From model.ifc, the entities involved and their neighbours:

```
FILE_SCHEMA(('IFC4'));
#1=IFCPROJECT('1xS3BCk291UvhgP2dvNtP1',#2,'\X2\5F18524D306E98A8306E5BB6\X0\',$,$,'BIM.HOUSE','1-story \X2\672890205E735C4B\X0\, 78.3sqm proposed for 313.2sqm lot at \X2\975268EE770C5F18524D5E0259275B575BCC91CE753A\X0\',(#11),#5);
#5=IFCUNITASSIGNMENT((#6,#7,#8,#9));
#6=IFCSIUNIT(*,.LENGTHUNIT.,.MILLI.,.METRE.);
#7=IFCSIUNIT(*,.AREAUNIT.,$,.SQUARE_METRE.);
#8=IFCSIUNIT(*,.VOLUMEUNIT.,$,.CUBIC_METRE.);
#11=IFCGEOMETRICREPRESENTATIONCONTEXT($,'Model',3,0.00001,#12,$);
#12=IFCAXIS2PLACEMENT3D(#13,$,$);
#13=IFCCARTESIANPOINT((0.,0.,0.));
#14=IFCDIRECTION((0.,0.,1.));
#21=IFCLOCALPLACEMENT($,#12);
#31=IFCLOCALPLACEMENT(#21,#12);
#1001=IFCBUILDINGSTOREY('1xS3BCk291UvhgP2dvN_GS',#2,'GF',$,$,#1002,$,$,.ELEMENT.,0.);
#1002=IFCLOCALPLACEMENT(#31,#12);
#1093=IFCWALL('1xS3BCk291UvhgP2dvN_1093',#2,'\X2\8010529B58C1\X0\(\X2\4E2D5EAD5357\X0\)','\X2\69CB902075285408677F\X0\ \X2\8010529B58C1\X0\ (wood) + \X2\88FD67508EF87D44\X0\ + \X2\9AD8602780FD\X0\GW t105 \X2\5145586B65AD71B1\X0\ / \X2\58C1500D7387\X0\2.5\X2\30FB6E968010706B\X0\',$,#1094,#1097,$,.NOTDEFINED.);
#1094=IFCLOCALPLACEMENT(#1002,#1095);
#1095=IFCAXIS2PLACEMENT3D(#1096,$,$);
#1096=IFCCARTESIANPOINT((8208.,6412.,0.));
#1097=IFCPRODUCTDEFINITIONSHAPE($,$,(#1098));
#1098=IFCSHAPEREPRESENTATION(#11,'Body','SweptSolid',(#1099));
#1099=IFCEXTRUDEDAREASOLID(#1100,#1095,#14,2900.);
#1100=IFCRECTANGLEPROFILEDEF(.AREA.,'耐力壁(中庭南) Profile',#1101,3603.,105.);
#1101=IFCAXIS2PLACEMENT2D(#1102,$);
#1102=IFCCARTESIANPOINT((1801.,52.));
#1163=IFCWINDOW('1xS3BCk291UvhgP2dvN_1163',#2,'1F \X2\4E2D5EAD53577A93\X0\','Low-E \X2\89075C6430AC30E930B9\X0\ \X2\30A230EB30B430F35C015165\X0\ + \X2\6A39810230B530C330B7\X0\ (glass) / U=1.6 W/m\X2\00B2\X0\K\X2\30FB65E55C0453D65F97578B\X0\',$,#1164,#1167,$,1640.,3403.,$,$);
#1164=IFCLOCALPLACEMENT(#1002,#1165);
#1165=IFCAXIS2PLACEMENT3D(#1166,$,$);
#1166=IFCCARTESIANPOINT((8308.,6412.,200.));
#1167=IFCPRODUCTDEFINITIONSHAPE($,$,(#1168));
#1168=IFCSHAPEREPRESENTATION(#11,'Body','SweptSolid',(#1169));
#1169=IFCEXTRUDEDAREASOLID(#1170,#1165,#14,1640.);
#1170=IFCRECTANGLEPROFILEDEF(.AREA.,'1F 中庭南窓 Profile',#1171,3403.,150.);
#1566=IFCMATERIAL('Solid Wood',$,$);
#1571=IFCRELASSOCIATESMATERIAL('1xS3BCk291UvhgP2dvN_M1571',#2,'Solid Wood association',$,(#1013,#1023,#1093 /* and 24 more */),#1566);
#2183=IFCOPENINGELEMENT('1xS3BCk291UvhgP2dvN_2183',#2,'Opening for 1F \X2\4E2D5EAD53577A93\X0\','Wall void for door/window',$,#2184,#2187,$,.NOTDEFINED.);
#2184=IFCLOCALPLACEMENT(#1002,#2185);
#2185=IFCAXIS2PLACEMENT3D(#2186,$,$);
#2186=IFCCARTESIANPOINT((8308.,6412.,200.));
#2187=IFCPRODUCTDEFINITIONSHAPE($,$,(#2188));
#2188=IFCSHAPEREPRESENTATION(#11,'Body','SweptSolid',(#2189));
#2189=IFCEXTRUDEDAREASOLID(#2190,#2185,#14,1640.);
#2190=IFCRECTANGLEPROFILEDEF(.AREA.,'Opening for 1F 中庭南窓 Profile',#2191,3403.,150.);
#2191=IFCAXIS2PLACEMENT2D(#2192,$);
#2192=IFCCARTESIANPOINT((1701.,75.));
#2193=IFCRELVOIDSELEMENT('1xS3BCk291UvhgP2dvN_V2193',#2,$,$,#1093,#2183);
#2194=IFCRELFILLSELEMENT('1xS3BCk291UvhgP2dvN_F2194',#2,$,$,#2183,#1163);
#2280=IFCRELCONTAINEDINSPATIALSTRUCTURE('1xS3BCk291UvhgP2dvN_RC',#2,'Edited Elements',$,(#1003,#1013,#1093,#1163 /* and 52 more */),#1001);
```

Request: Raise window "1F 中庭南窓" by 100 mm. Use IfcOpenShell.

```python
import numpy as np
import ifcopenshell
import ifcopenshell.api.geometry
import ifcopenshell.util.placement
import ifcopenshell.util.unit

model = ifcopenshell.open("model.ifc")
unit_scale = ifcopenshell.util.unit.calculate_unit_scale(model)

window = model.by_guid("1xS3BCk291UvhgP2dvN_1163")
opening = window.FillsVoids[0].RelatingOpeningElement
dz = 100.0

shift = np.array([0.0, 0.0, dz])
# The window is not placed relative to its opening, so move both.
for product in (opening, window):
    matrix = ifcopenshell.util.placement.get_local_placement(product.ObjectPlacement)
    matrix[:3, 3] += shift
    ifcopenshell.api.geometry.edit_object_placement(model, product=product, matrix=matrix, is_si=False)

print(f"moved by {dz * unit_scale:+.3f} m")

model.write("model_updated.ifc")
```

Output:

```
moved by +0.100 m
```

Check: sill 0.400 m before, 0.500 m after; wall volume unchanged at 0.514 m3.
